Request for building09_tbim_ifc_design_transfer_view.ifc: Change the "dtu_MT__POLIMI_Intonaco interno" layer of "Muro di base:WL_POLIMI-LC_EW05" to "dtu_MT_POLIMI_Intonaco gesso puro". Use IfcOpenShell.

First a look at what the model holds.

```python
import ifcopenshell
import ifcopenshell.util.element

model = ifcopenshell.open("building09_tbim_ifc_design_transfer_view.ifc")
print(model.schema)
for layer_set in model.by_type("IfcMaterialLayerSet"):
    if layer_set.LayerSetName == "Muro di base:WL_POLIMI-LC_EW05":
        for layer in layer_set.MaterialLayers:
            print(layer.id(), layer.Material and layer.Material.Name, layer.LayerThickness, sep=" | ")
        print(len(ifcopenshell.util.element.get_elements_by_material(model, layer_set)), "elements and types use it")
print(sorted(m.Name for m in model.by_type("IfcMaterial") if m.Name)[:60])
```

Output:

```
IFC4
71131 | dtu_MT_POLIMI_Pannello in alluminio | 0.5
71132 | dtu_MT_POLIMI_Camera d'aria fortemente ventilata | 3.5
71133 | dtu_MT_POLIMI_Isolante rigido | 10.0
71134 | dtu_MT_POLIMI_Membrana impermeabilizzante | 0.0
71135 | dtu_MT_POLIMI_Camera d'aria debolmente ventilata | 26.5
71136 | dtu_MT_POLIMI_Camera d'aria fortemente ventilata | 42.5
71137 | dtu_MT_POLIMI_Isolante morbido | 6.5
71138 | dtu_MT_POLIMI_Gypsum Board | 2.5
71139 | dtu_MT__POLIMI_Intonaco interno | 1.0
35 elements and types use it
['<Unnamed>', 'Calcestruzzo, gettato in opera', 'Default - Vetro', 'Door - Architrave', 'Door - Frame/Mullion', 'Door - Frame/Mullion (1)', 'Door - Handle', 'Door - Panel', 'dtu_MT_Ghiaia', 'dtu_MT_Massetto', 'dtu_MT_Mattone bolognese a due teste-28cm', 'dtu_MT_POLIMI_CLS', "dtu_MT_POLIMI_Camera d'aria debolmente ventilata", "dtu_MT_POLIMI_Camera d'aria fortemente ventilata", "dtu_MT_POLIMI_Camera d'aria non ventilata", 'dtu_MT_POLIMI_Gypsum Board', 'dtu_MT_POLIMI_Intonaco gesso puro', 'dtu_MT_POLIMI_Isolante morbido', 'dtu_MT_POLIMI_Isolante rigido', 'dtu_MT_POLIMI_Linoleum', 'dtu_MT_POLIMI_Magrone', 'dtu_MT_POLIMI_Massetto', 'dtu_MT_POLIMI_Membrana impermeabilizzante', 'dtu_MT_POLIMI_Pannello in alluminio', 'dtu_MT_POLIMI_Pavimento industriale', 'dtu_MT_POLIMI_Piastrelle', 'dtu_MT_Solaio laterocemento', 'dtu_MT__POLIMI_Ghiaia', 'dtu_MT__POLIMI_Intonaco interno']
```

```python
import ifcopenshell
import ifcopenshell.api.material

model = ifcopenshell.open("building09_tbim_ifc_design_transfer_view.ifc")

layer_set = next(s for s in model.by_type("IfcMaterialLayerSet") if s.LayerSetName == "Muro di base:WL_POLIMI-LC_EW05")
layer = next(l for l in layer_set.MaterialLayers if l.Material and l.Material.Name == "dtu_MT__POLIMI_Intonaco interno")
material = next(m for m in model.by_type("IfcMaterial") if m.Name == "dtu_MT_POLIMI_Intonaco gesso puro")

# Point this one layer at the other material; renaming the old one would change it everywhere.
ifcopenshell.api.material.edit_layer(model, layer=layer, attributes={"Name": material.Name}, material=material)

print([l.Material.Name if l.Material else None for l in layer_set.MaterialLayers])

model.write("building09_tbim_ifc_design_transfer_view_updated.ifc")
```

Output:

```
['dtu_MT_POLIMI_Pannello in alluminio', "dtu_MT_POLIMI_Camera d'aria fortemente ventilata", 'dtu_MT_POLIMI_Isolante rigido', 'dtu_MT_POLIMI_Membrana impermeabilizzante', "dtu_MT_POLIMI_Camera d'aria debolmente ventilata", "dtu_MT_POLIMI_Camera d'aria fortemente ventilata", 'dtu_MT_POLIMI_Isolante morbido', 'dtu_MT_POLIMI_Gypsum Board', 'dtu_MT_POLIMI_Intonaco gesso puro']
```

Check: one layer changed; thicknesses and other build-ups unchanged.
